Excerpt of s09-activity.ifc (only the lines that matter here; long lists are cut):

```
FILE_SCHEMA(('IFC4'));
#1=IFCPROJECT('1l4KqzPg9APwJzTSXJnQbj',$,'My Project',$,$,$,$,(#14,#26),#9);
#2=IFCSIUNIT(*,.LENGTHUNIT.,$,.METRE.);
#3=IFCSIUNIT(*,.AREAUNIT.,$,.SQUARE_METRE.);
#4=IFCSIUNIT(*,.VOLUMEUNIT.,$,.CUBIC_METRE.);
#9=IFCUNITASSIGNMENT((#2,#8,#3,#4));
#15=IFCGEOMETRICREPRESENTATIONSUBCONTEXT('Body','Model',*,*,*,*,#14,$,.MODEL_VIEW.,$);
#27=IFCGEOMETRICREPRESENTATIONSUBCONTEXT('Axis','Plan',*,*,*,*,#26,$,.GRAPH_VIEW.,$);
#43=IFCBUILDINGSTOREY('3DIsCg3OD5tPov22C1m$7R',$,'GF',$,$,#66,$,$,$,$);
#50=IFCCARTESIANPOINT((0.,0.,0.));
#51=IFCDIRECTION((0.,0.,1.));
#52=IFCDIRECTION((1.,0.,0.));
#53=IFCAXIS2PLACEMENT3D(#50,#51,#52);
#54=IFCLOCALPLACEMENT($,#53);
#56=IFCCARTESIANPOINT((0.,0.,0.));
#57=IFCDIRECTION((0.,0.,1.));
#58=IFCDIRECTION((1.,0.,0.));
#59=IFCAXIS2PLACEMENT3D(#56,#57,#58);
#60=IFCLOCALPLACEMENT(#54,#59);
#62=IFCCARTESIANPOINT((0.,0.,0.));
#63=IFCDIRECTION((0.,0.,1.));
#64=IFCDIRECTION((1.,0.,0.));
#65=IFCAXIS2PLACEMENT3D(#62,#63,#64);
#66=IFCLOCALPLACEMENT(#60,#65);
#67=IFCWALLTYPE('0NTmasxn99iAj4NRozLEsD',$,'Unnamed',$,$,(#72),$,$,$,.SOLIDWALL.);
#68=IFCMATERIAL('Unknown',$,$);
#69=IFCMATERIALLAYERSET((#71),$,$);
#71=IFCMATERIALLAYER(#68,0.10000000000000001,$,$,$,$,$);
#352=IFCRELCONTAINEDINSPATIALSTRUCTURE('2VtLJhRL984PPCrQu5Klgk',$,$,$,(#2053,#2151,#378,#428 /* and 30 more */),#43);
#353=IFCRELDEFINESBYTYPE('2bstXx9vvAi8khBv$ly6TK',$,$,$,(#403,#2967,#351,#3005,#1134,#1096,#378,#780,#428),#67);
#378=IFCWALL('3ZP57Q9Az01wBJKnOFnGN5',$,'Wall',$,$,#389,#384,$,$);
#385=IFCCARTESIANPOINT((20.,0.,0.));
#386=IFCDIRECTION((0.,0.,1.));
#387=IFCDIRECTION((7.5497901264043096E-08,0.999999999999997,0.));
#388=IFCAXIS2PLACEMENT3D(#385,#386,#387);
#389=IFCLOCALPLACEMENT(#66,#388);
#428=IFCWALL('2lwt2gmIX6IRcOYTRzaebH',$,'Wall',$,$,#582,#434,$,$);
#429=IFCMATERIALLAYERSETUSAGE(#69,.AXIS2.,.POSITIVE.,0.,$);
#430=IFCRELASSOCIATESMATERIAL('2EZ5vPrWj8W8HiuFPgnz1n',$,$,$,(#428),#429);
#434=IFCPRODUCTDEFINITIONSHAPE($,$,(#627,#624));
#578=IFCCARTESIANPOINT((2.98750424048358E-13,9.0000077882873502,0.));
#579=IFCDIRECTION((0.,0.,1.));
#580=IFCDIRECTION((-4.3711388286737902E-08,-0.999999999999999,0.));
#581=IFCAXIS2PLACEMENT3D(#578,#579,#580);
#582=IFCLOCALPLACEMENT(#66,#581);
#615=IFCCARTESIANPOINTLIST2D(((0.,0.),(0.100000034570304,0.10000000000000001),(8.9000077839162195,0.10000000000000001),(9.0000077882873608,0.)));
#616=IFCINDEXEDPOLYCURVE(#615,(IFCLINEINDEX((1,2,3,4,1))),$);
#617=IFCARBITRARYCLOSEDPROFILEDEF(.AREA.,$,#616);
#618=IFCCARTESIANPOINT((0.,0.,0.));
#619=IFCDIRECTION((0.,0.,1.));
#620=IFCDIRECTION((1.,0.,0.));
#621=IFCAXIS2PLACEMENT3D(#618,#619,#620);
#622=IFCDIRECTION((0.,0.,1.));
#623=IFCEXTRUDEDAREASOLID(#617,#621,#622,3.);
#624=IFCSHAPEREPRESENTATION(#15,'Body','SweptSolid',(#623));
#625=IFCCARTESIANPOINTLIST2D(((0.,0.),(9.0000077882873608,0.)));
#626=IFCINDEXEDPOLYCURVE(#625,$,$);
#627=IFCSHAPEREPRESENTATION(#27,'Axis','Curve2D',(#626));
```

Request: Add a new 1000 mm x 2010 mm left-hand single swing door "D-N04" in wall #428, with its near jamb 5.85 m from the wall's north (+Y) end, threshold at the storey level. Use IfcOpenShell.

```python
import numpy as np
import ifcopenshell
import ifcopenshell.api.feature
import ifcopenshell.api.geometry
import ifcopenshell.api.root
import ifcopenshell.api.spatial
import ifcopenshell.geom
import ifcopenshell.util.element
import ifcopenshell.util.placement
import ifcopenshell.util.representation
import ifcopenshell.util.shape
import ifcopenshell.util.unit

model = ifcopenshell.open("s09-activity.ifc")
unit_scale = ifcopenshell.util.unit.calculate_unit_scale(model)
settings = ifcopenshell.geom.settings()


def volume(element):
    """Net volume in cubic metres, openings subtracted."""
    shape = ifcopenshell.geom.create_shape(settings, element)
    return ifcopenshell.util.shape.get_volume(shape.geometry)


wall = model.by_guid("2lwt2gmIX6IRcOYTRzaebH")
storey = ifcopenshell.util.element.get_container(wall, ifc_class="IfcBuildingStorey")
context = ifcopenshell.util.representation.get_context(model, "Model", "Body", "MODEL_VIEW")
before = volume(wall)

width, height, from_end, sill = 1, 2.01, 5.85, 0.0  # metres

# The wall runs along its own X axis, and the end named is its -X end.
wall_shape = ifcopenshell.geom.create_shape(settings, wall)
x, y, z = ifcopenshell.util.shape.get_vertices(wall_shape.geometry).T
start = x.min() + from_end
face, thickness = float(y.min()), float(y.max() - y.min())
wall_matrix = ifcopenshell.util.placement.get_local_placement(wall.ObjectPlacement)
level = ifcopenshell.util.placement.get_local_placement(storey.ObjectPlacement)[2, 3]


def in_wall(x, y):
    """Placement at x, y metres in the wall's axes, at sill height."""
    matrix = wall_matrix.copy()
    matrix[:, 3] = wall_matrix @ np.array([x / unit_scale, y / unit_scale, 0.0, 1.0])
    matrix[2, 3] = level + sill / unit_scale
    return matrix


# Opening: a box that overshoots both wall faces by 50 mm.
opening = ifcopenshell.api.root.create_entity(model, ifc_class="IfcOpeningElement", predefined_type="OPENING")
box = ifcopenshell.api.geometry.add_wall_representation(
    model, context=context, length=width, height=height, thickness=thickness + 0.1
)
ifcopenshell.api.geometry.assign_representation(model, product=opening, representation=box)
ifcopenshell.api.geometry.edit_object_placement(model, product=opening, matrix=in_wall(start, face - 0.05), is_si=False)
ifcopenshell.api.feature.add_feature(model, feature=opening, element=wall)

door = ifcopenshell.api.root.create_entity(model, ifc_class="IfcDoor", name="D-N04", predefined_type="DOOR")
door.OverallWidth, door.OverallHeight = width / unit_scale, height / unit_scale
door.OperationType = "SINGLE_SWING_LEFT"
body = ifcopenshell.api.geometry.add_door_representation(
    model,
    context=context,
    overall_width=door.OverallWidth,
    overall_height=door.OverallHeight,
    operation_type="SINGLE_SWING_LEFT",
    lining_properties={"LiningDepth": thickness / unit_scale, "ThresholdDepth": thickness / unit_scale},
)
ifcopenshell.api.geometry.assign_representation(model, product=door, representation=body)
ifcopenshell.api.spatial.assign_container(model, products=[door], relating_structure=storey)
ifcopenshell.api.feature.add_filling(model, opening=opening, element=door)

# The lining spans the wall, so the door starts at the wall face.
ifcopenshell.api.geometry.edit_object_placement(model, product=door, matrix=in_wall(start, face), is_si=False)

after = volume(wall)

print(f"wall volume {before:.3f} -> {after:.3f} m3")

model.write("s09-activity-out.ifc")
```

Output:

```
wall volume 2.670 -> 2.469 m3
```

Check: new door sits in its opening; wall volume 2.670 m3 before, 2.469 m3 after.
